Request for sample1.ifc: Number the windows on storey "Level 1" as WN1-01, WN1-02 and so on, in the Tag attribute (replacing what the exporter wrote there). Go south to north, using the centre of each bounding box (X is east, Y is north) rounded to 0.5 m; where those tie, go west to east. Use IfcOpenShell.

First a look at what the model holds.

```python
import ifcopenshell
import ifcopenshell.util.element
import ifcopenshell.util.placement

model = ifcopenshell.open("sample1.ifc")
print(model.schema)
storey = next(s for s in model.by_type("IfcBuildingStorey") if s.Name == "Level 1")
windows = [e for e in ifcopenshell.util.element.get_decomposition(storey) if e.is_a("IfcWindow")]
for e in sorted(windows, key=lambda e: e.id()):
    origin = ifcopenshell.util.placement.get_local_placement(e.ObjectPlacement)[:3, 3]
    print(e.id(), e.Tag, e.Name, origin.round(2) + 0.0, sep=" | ")
```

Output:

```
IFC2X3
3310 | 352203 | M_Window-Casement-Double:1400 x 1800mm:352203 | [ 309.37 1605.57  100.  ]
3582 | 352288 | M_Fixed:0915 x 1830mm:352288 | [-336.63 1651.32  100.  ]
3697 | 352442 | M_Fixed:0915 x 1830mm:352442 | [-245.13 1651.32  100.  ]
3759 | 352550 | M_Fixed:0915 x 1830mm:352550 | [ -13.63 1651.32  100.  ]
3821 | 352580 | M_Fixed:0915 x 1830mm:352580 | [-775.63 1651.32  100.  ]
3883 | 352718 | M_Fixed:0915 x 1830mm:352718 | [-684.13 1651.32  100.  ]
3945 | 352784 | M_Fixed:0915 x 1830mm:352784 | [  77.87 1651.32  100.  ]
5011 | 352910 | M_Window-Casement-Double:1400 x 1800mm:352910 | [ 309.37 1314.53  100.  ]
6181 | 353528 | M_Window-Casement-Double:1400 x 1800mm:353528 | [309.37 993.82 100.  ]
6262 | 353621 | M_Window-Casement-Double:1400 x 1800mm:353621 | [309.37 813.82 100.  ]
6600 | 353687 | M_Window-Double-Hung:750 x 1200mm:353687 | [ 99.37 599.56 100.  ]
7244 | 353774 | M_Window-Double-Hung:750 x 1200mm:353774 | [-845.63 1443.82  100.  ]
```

```python
import ifcopenshell
import ifcopenshell.geom
import ifcopenshell.util.element
import ifcopenshell.util.shape

model = ifcopenshell.open("sample1.ifc")
settings = ifcopenshell.geom.settings()
settings.set("use-world-coords", True)


def centre(element):
    shape = ifcopenshell.geom.create_shape(settings, element)
    return ifcopenshell.util.shape.get_bbox_centroid(shape.geometry)


storey = next(s for s in model.by_type("IfcBuildingStorey") if s.Name == "Level 1")
windows = [e for e in ifcopenshell.util.element.get_decomposition(storey) if e.is_a("IfcWindow")]

# Insertion points can sit at a corner or the storey origin, so sort by the geometry (in metres).
centres = {e: centre(e) for e in windows}
windows.sort(key=lambda e: (round(centres[e][1] / 0.5), centres[e][0]))

for i, e in enumerate(windows, start=1):
    number = f"WN1-{i:02d}"
    e.Tag = number
    print(e.id(), number)

model.write("sample1_updated.ifc")
```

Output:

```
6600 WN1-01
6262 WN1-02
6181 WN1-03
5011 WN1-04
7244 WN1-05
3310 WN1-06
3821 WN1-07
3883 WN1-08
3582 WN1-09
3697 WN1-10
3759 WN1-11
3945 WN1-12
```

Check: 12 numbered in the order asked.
